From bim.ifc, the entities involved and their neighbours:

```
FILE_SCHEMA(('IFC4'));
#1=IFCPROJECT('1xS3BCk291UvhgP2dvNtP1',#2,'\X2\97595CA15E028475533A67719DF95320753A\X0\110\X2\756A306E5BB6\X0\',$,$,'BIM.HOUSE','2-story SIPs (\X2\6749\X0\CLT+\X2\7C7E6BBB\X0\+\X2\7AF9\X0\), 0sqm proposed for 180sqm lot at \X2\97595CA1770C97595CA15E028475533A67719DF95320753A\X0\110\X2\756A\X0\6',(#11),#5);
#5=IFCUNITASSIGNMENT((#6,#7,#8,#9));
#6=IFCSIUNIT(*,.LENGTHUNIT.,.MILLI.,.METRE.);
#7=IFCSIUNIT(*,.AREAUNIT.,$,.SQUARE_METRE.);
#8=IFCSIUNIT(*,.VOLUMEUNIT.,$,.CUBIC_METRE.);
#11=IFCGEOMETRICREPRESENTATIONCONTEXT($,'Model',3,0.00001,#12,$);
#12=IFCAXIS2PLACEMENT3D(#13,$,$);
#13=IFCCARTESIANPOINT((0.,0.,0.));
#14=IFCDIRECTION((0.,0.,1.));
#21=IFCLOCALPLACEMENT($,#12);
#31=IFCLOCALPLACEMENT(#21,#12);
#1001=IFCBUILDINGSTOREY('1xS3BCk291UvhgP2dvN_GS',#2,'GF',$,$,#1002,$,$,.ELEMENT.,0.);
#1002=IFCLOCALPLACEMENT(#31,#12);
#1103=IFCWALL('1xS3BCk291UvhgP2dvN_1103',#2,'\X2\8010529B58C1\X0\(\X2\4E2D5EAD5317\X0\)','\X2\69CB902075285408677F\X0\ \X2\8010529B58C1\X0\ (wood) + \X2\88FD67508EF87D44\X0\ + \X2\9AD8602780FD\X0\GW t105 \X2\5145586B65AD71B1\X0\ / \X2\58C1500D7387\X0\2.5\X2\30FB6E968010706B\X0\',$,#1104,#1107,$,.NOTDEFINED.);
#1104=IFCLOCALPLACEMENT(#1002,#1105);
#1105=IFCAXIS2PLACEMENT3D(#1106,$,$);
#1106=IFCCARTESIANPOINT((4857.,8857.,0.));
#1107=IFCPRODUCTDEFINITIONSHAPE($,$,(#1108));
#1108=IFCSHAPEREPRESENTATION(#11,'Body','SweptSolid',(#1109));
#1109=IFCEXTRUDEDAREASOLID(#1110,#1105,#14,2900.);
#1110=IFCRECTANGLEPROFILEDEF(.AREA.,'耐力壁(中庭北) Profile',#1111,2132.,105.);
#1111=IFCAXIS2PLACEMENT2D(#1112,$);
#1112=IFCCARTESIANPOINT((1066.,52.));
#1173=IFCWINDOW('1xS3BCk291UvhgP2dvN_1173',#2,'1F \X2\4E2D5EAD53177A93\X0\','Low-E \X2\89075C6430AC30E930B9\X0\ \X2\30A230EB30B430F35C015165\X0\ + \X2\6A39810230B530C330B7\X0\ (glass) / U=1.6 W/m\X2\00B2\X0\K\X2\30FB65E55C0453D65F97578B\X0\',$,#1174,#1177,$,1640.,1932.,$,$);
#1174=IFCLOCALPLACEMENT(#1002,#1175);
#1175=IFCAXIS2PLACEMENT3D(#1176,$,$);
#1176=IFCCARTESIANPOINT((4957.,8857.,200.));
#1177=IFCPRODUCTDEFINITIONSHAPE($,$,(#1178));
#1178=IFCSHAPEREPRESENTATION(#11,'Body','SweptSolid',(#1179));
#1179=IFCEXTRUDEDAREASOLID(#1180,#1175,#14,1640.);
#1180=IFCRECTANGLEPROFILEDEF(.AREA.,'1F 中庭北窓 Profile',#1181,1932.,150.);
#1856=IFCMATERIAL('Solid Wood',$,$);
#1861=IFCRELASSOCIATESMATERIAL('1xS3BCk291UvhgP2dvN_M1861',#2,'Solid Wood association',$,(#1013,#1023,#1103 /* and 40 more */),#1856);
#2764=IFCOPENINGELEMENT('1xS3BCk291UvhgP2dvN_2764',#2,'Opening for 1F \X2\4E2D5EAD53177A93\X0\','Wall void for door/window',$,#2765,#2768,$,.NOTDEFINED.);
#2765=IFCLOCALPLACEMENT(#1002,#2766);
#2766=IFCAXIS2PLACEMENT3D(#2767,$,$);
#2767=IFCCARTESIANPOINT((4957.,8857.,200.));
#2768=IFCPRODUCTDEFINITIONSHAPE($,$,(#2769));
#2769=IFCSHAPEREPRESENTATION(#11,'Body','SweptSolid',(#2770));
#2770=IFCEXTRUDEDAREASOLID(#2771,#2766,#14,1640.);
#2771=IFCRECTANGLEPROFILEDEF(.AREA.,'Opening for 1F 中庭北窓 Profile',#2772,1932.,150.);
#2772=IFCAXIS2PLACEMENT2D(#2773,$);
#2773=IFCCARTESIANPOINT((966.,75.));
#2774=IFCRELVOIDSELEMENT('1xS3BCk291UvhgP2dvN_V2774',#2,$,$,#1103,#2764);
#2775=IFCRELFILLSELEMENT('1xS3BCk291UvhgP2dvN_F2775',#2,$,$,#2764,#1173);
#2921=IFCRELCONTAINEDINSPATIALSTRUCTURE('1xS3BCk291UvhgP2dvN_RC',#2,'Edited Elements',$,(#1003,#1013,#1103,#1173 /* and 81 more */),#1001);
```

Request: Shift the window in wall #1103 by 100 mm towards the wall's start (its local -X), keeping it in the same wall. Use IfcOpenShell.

```python
import ifcopenshell
import ifcopenshell.api.geometry
import ifcopenshell.util.placement
import ifcopenshell.util.unit

model = ifcopenshell.open("bim.ifc")
unit_scale = ifcopenshell.util.unit.calculate_unit_scale(model)

window = model.by_guid("1xS3BCk291UvhgP2dvN_1173")
opening = window.FillsVoids[0].RelatingOpeningElement
wall = opening.VoidsElements[0].RelatingBuildingElement

wall_matrix = ifcopenshell.util.placement.get_local_placement(wall.ObjectPlacement)
shift = wall_matrix[:3, 0] * -0.1 / unit_scale
before = ifcopenshell.util.placement.get_local_placement(window.ObjectPlacement)[:3, 3].copy()

# The window is not placed relative to its opening, so move both.
for product in (opening, window):
    matrix = ifcopenshell.util.placement.get_local_placement(product.ObjectPlacement)
    matrix[:3, 3] += shift
    ifcopenshell.api.geometry.edit_object_placement(model, product=product, matrix=matrix, is_si=False)

after = ifcopenshell.util.placement.get_local_placement(window.ObjectPlacement)[:3, 3]
print("window moved by", (after - before).round(3) + 0.0)

model.write("bim_edited.ifc")
```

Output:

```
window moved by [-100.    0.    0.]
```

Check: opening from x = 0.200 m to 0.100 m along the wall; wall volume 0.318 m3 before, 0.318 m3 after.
